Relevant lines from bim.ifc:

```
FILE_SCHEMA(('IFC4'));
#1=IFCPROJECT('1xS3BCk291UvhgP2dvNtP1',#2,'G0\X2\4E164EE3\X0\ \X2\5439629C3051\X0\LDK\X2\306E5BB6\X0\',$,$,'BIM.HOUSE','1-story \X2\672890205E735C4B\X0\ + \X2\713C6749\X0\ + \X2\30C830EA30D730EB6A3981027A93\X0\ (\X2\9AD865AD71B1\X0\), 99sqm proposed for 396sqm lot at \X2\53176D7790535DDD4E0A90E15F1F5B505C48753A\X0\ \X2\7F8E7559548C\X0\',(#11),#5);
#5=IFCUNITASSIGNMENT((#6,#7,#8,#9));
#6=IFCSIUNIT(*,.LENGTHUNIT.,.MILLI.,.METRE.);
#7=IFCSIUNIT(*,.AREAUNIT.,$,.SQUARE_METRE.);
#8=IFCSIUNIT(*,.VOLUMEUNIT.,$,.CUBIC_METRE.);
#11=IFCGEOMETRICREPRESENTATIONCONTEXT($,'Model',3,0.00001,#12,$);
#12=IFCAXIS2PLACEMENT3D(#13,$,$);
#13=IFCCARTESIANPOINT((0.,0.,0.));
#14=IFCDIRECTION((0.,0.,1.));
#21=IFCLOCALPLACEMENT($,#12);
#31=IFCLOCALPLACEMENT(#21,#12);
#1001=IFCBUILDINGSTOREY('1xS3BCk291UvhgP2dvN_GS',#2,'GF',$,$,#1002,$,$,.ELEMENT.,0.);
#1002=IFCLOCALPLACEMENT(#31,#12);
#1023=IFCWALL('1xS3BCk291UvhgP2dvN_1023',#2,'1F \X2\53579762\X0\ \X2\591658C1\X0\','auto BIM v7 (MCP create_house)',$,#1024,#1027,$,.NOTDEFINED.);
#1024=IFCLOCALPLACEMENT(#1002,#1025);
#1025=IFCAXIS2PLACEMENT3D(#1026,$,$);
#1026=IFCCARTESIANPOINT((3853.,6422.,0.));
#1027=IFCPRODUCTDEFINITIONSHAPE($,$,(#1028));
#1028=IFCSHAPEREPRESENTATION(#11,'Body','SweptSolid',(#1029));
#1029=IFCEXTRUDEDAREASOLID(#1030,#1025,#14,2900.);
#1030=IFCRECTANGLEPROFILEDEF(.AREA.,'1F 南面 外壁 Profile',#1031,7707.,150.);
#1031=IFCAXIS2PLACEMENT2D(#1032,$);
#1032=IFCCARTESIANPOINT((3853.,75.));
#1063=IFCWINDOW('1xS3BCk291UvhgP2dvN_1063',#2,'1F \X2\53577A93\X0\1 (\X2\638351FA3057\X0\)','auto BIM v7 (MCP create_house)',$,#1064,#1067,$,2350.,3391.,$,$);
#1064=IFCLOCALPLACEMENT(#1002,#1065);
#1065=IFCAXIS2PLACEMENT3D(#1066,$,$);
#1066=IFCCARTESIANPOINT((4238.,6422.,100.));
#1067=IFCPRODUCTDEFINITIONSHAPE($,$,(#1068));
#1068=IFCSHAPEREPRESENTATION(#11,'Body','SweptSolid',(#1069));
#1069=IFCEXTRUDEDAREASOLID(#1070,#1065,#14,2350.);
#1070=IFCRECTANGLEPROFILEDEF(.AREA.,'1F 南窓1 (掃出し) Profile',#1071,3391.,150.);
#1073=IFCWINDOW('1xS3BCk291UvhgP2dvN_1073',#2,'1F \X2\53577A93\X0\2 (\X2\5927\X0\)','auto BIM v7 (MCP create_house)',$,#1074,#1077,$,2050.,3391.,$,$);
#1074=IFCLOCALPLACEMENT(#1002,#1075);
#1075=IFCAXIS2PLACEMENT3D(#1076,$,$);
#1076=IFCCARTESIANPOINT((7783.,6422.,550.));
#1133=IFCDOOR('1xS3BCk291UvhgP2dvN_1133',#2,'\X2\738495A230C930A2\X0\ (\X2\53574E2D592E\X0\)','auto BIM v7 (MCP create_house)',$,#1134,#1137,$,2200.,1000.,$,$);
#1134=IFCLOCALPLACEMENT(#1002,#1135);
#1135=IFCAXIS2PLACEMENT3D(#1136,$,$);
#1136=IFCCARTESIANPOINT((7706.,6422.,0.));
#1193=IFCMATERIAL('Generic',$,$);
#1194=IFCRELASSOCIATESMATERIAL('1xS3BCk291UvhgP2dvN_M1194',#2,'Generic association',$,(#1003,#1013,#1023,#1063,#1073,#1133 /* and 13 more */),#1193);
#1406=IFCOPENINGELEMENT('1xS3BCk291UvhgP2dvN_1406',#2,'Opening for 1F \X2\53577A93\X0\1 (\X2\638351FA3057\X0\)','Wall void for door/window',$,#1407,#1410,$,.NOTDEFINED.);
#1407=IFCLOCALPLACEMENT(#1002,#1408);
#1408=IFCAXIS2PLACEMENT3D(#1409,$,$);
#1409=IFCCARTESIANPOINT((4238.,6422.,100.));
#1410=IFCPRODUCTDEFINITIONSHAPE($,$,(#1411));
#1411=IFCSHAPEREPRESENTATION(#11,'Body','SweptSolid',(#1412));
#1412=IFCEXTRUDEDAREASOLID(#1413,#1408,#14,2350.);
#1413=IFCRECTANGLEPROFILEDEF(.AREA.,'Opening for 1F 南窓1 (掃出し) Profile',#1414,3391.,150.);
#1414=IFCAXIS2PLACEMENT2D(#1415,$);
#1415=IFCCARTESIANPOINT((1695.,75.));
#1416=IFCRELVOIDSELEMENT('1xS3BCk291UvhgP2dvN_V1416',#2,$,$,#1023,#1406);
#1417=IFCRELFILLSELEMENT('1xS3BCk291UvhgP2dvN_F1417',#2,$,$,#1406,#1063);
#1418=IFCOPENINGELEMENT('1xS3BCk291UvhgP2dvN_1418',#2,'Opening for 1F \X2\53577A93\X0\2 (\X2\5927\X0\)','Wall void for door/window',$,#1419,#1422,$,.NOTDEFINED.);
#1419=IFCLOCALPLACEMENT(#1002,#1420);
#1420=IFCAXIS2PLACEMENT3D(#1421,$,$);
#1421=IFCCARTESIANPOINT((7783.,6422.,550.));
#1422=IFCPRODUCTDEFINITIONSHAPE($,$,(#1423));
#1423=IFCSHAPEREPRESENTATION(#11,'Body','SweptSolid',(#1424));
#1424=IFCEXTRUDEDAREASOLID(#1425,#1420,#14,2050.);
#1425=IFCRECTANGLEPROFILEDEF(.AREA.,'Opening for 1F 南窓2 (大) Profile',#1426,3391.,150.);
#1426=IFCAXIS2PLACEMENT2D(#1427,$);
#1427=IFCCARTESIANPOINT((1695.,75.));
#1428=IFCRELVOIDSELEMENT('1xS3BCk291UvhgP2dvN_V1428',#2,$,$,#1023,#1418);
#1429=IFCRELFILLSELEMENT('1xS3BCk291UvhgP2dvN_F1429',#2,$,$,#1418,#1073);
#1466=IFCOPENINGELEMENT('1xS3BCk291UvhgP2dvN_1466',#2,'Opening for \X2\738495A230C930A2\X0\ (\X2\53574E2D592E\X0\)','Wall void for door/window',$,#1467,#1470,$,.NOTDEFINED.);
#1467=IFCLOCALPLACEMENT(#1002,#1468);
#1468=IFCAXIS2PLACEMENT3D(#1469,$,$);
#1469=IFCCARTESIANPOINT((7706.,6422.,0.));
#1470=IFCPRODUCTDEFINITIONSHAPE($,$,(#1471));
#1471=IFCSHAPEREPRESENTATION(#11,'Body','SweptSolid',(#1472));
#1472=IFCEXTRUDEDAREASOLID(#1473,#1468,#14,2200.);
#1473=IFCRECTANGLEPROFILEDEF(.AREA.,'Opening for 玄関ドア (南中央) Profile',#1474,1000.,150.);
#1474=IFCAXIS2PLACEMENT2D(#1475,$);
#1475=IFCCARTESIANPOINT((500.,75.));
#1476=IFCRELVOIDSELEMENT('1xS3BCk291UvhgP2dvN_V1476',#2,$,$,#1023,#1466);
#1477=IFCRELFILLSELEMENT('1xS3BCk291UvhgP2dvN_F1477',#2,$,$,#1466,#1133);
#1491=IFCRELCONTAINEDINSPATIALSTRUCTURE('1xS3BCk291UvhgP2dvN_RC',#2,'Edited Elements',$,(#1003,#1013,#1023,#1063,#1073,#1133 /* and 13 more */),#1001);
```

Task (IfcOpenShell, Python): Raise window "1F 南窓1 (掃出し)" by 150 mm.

```python
import numpy as np
import ifcopenshell
import ifcopenshell.api.geometry
import ifcopenshell.util.placement
import ifcopenshell.util.unit

model = ifcopenshell.open("bim.ifc")
unit_scale = ifcopenshell.util.unit.calculate_unit_scale(model)

window = model.by_id(1063)
opening = window.FillsVoids[0].RelatingOpeningElement
dz = 150.0

shift = np.array([0.0, 0.0, dz])
# The window is not placed relative to its opening, so move both.
for product in (opening, window):
    matrix = ifcopenshell.util.placement.get_local_placement(product.ObjectPlacement)
    matrix[:3, 3] += shift
    ifcopenshell.api.geometry.edit_object_placement(model, product=product, matrix=matrix, is_si=False)

print(f"moved by {dz * unit_scale:+.3f} m")

model.write("bim_edited.ifc")
```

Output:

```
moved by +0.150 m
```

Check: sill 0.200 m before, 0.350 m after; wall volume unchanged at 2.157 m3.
